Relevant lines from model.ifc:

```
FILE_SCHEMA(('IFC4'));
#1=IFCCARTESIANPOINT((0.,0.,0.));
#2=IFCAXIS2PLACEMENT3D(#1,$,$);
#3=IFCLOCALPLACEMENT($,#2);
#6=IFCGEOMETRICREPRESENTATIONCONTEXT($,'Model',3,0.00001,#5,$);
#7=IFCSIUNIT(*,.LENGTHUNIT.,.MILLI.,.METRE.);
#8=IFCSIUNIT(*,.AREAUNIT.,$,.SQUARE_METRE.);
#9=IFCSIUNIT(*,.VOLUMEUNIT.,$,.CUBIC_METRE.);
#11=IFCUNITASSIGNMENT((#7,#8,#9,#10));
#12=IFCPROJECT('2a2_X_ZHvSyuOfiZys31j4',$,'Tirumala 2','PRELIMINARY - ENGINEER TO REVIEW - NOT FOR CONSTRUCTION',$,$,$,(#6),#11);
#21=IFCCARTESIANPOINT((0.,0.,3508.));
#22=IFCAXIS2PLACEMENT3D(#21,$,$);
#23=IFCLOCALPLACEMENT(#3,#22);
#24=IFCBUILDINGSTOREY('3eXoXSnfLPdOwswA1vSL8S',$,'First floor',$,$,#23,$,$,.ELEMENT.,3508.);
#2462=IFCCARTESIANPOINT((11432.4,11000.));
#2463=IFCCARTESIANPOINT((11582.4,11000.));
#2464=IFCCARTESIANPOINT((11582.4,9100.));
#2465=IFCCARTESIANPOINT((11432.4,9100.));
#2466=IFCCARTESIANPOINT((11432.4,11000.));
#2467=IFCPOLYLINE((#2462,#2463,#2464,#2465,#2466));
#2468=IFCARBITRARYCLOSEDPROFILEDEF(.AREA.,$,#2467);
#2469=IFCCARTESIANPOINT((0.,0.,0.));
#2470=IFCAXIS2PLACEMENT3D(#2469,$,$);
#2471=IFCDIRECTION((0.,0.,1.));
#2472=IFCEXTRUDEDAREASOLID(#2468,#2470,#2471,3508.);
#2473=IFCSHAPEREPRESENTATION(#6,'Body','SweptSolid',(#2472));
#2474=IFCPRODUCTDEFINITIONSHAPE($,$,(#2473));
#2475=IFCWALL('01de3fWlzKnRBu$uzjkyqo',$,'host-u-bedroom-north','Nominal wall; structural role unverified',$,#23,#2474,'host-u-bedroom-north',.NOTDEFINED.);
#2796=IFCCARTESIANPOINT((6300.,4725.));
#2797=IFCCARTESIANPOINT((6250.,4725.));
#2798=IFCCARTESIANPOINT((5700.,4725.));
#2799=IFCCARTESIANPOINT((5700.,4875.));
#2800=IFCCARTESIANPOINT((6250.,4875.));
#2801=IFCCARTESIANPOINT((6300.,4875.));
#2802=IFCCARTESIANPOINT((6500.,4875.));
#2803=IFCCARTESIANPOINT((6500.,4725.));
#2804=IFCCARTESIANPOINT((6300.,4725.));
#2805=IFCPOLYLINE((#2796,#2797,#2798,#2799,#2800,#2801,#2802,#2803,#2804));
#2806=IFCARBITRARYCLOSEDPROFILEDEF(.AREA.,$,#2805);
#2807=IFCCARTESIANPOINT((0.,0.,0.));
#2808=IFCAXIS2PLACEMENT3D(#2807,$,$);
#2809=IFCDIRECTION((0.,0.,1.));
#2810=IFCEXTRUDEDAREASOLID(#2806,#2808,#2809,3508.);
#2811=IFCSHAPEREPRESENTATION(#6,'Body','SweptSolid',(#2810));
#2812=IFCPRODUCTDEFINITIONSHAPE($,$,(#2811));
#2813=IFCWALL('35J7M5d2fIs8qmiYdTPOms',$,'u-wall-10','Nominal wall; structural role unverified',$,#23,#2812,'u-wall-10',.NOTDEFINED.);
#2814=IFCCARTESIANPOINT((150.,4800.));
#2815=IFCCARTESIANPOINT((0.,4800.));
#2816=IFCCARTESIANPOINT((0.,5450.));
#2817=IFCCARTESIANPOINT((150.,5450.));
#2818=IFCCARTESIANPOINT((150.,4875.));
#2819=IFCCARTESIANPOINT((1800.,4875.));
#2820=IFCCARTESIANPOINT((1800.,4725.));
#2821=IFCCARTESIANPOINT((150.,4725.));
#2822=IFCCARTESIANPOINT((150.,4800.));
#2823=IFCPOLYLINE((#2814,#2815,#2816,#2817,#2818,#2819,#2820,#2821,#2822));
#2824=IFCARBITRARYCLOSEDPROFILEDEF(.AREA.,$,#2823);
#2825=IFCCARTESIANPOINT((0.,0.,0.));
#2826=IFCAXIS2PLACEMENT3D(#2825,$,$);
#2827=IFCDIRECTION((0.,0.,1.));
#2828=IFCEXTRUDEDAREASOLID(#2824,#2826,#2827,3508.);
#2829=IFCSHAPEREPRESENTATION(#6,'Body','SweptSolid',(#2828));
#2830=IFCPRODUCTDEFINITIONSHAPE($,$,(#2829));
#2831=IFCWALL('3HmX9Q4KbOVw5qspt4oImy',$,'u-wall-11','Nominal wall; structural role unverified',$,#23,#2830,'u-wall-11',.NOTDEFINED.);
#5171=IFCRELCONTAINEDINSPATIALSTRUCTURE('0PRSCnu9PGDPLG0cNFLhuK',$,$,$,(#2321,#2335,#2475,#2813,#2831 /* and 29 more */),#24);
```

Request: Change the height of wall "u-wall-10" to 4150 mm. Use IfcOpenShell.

```python
import ifcopenshell
import ifcopenshell.geom
import ifcopenshell.util.shape
import ifcopenshell.util.unit

model = ifcopenshell.open("model.ifc")
unit_scale = ifcopenshell.util.unit.calculate_unit_scale(model)
settings = ifcopenshell.geom.settings()


def volume(element):
    """Net volume in cubic metres, openings subtracted."""
    shape = ifcopenshell.geom.create_shape(settings, element)
    return ifcopenshell.util.shape.get_volume(shape.geometry)


wall = model.by_id(2813)
before = volume(wall)

body = next(r for r in wall.Representation.Representations if r.RepresentationIdentifier == "Body")
solid = body.Items[0]
old_height = solid.Depth
solid.Depth = 4.15 / unit_scale
after = volume(wall)

print(f"height {old_height:g} -> {solid.Depth:g}, volume {before:.3f} -> {after:.3f} m3")

model.write("model_rev.ifc")
```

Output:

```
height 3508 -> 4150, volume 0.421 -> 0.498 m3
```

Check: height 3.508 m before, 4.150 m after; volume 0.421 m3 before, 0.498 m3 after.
